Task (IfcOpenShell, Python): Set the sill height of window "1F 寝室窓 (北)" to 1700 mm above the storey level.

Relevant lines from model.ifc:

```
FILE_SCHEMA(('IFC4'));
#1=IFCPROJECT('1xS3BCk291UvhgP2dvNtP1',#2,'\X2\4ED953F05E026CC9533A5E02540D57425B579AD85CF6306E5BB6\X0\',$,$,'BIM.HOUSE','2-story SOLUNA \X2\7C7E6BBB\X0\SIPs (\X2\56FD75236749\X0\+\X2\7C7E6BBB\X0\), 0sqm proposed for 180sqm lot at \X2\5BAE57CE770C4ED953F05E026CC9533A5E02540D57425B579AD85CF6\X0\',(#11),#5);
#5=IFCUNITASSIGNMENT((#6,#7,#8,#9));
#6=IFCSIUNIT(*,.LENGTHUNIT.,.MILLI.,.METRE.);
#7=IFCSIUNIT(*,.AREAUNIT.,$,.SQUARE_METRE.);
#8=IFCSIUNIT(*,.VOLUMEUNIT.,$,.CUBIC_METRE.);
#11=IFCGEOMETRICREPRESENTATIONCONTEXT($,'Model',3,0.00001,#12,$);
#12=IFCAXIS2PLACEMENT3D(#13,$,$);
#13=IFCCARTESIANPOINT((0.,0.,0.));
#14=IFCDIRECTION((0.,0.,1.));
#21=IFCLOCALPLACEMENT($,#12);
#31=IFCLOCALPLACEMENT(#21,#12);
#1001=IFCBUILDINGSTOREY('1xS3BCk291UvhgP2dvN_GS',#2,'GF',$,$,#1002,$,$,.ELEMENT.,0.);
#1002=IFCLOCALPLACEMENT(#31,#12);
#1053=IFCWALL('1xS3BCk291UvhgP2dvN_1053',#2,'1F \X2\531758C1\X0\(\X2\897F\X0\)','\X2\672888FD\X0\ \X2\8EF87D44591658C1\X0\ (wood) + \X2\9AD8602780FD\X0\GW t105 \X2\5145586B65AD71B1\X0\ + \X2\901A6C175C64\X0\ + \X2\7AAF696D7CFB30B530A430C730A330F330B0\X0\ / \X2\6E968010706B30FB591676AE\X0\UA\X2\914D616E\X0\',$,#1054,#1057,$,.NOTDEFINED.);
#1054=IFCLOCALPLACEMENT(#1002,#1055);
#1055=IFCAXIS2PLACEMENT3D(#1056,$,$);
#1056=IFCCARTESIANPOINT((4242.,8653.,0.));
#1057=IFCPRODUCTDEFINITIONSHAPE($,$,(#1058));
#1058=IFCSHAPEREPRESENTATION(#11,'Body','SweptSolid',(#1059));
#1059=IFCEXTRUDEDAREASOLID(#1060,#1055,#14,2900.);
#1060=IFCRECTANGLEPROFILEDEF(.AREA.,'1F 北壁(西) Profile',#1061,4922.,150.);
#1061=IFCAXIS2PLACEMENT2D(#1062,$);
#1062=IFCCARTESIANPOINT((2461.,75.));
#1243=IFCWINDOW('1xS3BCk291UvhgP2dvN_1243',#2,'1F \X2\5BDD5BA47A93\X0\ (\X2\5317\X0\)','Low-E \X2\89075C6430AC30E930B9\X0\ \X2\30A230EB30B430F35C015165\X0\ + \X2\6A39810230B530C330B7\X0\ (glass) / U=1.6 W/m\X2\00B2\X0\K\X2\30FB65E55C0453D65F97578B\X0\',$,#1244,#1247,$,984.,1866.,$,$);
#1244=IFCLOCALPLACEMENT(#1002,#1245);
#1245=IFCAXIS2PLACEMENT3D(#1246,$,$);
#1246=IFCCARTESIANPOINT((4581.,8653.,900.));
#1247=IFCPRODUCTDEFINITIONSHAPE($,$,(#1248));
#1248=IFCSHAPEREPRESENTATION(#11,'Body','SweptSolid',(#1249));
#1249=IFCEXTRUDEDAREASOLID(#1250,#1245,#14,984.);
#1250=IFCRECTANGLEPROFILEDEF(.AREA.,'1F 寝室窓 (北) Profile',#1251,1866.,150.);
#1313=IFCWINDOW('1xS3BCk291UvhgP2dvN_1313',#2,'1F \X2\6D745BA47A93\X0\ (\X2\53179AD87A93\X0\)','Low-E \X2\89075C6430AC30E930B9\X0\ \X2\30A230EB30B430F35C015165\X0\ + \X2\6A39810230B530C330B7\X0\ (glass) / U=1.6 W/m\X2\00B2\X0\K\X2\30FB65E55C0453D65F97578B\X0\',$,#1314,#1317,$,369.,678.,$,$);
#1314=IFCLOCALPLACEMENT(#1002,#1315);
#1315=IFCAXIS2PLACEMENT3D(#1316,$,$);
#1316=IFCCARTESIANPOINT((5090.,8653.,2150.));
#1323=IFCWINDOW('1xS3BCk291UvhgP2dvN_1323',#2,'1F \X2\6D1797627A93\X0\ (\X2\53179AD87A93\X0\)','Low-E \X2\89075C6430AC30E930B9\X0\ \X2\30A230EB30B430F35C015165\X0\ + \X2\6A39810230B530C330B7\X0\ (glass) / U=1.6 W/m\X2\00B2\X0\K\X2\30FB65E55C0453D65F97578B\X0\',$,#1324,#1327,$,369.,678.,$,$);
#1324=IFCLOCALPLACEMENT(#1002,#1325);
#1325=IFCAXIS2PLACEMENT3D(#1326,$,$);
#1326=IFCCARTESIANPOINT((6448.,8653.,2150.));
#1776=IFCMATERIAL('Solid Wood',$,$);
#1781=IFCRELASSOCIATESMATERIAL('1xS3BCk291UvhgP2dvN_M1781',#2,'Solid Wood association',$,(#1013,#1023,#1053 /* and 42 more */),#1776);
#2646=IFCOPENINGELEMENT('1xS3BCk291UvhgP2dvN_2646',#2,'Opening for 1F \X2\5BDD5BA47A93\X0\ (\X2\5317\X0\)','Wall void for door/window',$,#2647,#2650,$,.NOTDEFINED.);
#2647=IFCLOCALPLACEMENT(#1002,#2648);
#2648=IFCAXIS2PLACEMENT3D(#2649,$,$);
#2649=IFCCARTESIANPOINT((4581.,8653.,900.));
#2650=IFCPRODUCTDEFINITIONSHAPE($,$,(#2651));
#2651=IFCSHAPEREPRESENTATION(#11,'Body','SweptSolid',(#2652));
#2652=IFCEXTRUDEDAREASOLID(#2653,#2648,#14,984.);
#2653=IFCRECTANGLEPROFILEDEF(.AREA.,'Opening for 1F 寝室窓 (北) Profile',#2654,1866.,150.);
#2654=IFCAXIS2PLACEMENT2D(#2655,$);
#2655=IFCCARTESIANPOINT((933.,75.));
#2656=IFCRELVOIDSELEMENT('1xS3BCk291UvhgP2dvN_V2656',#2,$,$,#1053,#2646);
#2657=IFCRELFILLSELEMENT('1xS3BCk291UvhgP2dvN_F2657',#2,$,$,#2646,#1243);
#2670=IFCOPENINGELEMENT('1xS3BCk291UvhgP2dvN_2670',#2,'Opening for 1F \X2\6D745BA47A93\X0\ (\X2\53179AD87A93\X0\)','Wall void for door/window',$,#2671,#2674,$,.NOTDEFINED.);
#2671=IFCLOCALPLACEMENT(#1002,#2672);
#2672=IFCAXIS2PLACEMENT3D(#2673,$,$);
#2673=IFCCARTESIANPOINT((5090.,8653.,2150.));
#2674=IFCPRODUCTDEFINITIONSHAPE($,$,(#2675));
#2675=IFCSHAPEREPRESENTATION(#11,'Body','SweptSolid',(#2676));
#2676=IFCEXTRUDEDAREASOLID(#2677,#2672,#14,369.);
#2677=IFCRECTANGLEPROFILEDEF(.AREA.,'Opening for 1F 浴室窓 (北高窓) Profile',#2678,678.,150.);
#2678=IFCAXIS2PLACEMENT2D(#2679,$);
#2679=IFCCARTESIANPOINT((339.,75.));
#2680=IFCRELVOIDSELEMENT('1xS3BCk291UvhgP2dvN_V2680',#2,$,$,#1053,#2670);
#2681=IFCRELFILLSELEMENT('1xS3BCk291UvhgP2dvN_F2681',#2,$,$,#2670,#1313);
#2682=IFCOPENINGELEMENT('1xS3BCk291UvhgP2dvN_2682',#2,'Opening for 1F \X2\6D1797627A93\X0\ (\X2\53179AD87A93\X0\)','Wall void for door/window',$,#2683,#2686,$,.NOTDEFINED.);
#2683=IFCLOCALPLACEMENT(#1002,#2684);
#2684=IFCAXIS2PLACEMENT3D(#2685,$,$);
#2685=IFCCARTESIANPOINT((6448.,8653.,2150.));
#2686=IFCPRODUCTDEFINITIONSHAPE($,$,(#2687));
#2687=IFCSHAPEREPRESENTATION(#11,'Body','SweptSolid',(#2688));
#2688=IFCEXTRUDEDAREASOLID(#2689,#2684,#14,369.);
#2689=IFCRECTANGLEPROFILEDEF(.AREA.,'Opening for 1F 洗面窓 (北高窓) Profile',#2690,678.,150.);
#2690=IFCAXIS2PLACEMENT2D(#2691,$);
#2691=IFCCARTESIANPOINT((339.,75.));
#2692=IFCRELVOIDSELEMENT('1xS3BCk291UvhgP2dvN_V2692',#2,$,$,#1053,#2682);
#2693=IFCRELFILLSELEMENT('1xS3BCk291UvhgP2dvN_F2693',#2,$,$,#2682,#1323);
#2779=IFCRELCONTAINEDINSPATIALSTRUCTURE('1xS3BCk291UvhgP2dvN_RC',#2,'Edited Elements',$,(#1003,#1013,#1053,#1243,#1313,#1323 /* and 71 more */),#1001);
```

```python
import numpy as np
import ifcopenshell
import ifcopenshell.api.geometry
import ifcopenshell.geom
import ifcopenshell.util.element
import ifcopenshell.util.placement
import ifcopenshell.util.shape
import ifcopenshell.util.unit

model = ifcopenshell.open("model.ifc")
unit_scale = ifcopenshell.util.unit.calculate_unit_scale(model)

window = model.by_guid("1xS3BCk291UvhgP2dvN_1243")
opening = window.FillsVoids[0].RelatingOpeningElement
storey = ifcopenshell.util.element.get_container(window, ifc_class="IfcBuildingStorey")
level = ifcopenshell.util.placement.get_local_placement(storey.ObjectPlacement)[2, 3]

# The opening's origin need not be at the sill, so measure its lowest point.
shape = ifcopenshell.geom.create_shape(ifcopenshell.geom.settings(), opening)
bottom = ifcopenshell.util.shape.get_shape_bottom_elevation(shape, shape.geometry) / unit_scale
dz = level + 1.7 / unit_scale - bottom

shift = np.array([0.0, 0.0, dz])
# The window is not placed relative to its opening, so move both.
for product in (opening, window):
    matrix = ifcopenshell.util.placement.get_local_placement(product.ObjectPlacement)
    matrix[:3, 3] += shift
    ifcopenshell.api.geometry.edit_object_placement(model, product=product, matrix=matrix, is_si=False)

print(f"moved by {dz * unit_scale:+.3f} m")

model.write("model_updated.ifc")
```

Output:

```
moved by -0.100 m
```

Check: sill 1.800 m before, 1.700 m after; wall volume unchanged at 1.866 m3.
